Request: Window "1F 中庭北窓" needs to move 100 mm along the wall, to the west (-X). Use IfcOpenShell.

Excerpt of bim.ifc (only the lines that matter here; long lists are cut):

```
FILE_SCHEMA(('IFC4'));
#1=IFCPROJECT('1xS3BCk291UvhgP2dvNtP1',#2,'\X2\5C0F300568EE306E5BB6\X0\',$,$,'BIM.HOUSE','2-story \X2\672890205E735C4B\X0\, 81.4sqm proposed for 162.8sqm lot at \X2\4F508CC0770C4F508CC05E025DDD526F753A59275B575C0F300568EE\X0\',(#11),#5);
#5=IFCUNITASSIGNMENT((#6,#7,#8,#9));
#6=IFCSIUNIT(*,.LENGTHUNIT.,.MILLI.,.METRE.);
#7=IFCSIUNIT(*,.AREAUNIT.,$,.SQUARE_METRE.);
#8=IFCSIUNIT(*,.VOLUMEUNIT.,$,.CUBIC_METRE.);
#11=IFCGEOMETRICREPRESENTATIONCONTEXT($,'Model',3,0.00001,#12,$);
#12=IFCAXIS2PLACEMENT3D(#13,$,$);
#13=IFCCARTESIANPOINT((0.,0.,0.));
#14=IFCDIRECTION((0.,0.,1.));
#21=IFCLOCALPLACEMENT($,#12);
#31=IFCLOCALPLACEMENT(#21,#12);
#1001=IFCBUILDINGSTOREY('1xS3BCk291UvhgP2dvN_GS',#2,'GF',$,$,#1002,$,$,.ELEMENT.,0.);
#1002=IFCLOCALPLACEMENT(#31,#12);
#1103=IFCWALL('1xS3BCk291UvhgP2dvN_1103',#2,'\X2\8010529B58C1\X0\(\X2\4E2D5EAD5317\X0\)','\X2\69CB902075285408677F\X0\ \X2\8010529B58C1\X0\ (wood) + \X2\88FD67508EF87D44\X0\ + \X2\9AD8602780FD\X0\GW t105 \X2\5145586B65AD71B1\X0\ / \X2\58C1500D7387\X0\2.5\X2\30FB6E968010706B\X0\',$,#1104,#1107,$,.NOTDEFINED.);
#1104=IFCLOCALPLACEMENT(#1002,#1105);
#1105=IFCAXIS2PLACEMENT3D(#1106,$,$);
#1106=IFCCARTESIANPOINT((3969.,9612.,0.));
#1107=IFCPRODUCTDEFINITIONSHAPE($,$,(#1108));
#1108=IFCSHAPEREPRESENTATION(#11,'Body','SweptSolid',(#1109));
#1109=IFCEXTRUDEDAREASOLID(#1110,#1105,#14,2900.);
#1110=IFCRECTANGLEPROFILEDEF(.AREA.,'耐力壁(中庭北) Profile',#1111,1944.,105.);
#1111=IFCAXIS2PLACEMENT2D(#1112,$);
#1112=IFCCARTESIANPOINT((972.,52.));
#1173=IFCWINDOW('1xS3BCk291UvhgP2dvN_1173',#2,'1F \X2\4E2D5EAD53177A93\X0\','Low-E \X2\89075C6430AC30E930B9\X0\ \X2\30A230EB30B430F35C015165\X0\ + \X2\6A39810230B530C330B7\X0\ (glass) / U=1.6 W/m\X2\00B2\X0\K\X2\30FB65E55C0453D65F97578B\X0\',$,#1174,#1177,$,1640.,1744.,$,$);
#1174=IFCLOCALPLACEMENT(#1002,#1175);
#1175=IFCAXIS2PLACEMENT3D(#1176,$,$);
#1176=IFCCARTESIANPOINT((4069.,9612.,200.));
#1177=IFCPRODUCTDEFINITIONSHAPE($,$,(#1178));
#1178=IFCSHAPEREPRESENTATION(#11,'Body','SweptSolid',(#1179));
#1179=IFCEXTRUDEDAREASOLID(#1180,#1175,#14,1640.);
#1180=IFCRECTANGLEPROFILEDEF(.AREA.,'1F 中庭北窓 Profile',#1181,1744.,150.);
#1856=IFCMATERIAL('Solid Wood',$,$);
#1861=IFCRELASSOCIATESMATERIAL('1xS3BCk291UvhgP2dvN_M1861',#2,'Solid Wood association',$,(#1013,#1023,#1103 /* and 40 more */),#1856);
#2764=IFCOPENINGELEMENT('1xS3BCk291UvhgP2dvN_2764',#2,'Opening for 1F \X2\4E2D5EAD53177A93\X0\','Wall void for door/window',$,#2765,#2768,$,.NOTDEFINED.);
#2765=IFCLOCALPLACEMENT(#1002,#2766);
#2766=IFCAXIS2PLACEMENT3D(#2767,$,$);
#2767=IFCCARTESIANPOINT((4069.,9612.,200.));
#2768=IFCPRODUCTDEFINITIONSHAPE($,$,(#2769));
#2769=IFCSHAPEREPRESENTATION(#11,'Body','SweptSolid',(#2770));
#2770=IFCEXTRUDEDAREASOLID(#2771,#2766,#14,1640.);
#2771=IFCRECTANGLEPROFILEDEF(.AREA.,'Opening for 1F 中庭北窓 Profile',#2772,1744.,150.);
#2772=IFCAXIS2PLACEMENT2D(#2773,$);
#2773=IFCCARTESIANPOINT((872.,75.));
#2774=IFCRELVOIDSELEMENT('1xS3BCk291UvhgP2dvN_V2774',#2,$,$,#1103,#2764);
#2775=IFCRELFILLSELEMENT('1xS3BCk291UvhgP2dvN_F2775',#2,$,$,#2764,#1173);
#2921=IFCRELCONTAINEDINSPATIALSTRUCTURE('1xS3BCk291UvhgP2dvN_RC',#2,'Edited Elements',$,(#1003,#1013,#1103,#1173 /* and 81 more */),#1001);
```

```python
import ifcopenshell
import ifcopenshell.api.geometry
import ifcopenshell.util.placement
import ifcopenshell.util.unit

model = ifcopenshell.open("bim.ifc")
unit_scale = ifcopenshell.util.unit.calculate_unit_scale(model)

window = model.by_guid("1xS3BCk291UvhgP2dvN_1173")
opening = window.FillsVoids[0].RelatingOpeningElement
wall = opening.VoidsElements[0].RelatingBuildingElement

wall_matrix = ifcopenshell.util.placement.get_local_placement(wall.ObjectPlacement)
shift = wall_matrix[:3, 0] * -0.1 / unit_scale
before = ifcopenshell.util.placement.get_local_placement(window.ObjectPlacement)[:3, 3].copy()

# The window is not placed relative to its opening, so move both.
for product in (opening, window):
    matrix = ifcopenshell.util.placement.get_local_placement(product.ObjectPlacement)
    matrix[:3, 3] += shift
    ifcopenshell.api.geometry.edit_object_placement(model, product=product, matrix=matrix, is_si=False)

after = ifcopenshell.util.placement.get_local_placement(window.ObjectPlacement)[:3, 3]
print("window moved by", (after - before).round(3) + 0.0)

model.write("bim-out.ifc")
```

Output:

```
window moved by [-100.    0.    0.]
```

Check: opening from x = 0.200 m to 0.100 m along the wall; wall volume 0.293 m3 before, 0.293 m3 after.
